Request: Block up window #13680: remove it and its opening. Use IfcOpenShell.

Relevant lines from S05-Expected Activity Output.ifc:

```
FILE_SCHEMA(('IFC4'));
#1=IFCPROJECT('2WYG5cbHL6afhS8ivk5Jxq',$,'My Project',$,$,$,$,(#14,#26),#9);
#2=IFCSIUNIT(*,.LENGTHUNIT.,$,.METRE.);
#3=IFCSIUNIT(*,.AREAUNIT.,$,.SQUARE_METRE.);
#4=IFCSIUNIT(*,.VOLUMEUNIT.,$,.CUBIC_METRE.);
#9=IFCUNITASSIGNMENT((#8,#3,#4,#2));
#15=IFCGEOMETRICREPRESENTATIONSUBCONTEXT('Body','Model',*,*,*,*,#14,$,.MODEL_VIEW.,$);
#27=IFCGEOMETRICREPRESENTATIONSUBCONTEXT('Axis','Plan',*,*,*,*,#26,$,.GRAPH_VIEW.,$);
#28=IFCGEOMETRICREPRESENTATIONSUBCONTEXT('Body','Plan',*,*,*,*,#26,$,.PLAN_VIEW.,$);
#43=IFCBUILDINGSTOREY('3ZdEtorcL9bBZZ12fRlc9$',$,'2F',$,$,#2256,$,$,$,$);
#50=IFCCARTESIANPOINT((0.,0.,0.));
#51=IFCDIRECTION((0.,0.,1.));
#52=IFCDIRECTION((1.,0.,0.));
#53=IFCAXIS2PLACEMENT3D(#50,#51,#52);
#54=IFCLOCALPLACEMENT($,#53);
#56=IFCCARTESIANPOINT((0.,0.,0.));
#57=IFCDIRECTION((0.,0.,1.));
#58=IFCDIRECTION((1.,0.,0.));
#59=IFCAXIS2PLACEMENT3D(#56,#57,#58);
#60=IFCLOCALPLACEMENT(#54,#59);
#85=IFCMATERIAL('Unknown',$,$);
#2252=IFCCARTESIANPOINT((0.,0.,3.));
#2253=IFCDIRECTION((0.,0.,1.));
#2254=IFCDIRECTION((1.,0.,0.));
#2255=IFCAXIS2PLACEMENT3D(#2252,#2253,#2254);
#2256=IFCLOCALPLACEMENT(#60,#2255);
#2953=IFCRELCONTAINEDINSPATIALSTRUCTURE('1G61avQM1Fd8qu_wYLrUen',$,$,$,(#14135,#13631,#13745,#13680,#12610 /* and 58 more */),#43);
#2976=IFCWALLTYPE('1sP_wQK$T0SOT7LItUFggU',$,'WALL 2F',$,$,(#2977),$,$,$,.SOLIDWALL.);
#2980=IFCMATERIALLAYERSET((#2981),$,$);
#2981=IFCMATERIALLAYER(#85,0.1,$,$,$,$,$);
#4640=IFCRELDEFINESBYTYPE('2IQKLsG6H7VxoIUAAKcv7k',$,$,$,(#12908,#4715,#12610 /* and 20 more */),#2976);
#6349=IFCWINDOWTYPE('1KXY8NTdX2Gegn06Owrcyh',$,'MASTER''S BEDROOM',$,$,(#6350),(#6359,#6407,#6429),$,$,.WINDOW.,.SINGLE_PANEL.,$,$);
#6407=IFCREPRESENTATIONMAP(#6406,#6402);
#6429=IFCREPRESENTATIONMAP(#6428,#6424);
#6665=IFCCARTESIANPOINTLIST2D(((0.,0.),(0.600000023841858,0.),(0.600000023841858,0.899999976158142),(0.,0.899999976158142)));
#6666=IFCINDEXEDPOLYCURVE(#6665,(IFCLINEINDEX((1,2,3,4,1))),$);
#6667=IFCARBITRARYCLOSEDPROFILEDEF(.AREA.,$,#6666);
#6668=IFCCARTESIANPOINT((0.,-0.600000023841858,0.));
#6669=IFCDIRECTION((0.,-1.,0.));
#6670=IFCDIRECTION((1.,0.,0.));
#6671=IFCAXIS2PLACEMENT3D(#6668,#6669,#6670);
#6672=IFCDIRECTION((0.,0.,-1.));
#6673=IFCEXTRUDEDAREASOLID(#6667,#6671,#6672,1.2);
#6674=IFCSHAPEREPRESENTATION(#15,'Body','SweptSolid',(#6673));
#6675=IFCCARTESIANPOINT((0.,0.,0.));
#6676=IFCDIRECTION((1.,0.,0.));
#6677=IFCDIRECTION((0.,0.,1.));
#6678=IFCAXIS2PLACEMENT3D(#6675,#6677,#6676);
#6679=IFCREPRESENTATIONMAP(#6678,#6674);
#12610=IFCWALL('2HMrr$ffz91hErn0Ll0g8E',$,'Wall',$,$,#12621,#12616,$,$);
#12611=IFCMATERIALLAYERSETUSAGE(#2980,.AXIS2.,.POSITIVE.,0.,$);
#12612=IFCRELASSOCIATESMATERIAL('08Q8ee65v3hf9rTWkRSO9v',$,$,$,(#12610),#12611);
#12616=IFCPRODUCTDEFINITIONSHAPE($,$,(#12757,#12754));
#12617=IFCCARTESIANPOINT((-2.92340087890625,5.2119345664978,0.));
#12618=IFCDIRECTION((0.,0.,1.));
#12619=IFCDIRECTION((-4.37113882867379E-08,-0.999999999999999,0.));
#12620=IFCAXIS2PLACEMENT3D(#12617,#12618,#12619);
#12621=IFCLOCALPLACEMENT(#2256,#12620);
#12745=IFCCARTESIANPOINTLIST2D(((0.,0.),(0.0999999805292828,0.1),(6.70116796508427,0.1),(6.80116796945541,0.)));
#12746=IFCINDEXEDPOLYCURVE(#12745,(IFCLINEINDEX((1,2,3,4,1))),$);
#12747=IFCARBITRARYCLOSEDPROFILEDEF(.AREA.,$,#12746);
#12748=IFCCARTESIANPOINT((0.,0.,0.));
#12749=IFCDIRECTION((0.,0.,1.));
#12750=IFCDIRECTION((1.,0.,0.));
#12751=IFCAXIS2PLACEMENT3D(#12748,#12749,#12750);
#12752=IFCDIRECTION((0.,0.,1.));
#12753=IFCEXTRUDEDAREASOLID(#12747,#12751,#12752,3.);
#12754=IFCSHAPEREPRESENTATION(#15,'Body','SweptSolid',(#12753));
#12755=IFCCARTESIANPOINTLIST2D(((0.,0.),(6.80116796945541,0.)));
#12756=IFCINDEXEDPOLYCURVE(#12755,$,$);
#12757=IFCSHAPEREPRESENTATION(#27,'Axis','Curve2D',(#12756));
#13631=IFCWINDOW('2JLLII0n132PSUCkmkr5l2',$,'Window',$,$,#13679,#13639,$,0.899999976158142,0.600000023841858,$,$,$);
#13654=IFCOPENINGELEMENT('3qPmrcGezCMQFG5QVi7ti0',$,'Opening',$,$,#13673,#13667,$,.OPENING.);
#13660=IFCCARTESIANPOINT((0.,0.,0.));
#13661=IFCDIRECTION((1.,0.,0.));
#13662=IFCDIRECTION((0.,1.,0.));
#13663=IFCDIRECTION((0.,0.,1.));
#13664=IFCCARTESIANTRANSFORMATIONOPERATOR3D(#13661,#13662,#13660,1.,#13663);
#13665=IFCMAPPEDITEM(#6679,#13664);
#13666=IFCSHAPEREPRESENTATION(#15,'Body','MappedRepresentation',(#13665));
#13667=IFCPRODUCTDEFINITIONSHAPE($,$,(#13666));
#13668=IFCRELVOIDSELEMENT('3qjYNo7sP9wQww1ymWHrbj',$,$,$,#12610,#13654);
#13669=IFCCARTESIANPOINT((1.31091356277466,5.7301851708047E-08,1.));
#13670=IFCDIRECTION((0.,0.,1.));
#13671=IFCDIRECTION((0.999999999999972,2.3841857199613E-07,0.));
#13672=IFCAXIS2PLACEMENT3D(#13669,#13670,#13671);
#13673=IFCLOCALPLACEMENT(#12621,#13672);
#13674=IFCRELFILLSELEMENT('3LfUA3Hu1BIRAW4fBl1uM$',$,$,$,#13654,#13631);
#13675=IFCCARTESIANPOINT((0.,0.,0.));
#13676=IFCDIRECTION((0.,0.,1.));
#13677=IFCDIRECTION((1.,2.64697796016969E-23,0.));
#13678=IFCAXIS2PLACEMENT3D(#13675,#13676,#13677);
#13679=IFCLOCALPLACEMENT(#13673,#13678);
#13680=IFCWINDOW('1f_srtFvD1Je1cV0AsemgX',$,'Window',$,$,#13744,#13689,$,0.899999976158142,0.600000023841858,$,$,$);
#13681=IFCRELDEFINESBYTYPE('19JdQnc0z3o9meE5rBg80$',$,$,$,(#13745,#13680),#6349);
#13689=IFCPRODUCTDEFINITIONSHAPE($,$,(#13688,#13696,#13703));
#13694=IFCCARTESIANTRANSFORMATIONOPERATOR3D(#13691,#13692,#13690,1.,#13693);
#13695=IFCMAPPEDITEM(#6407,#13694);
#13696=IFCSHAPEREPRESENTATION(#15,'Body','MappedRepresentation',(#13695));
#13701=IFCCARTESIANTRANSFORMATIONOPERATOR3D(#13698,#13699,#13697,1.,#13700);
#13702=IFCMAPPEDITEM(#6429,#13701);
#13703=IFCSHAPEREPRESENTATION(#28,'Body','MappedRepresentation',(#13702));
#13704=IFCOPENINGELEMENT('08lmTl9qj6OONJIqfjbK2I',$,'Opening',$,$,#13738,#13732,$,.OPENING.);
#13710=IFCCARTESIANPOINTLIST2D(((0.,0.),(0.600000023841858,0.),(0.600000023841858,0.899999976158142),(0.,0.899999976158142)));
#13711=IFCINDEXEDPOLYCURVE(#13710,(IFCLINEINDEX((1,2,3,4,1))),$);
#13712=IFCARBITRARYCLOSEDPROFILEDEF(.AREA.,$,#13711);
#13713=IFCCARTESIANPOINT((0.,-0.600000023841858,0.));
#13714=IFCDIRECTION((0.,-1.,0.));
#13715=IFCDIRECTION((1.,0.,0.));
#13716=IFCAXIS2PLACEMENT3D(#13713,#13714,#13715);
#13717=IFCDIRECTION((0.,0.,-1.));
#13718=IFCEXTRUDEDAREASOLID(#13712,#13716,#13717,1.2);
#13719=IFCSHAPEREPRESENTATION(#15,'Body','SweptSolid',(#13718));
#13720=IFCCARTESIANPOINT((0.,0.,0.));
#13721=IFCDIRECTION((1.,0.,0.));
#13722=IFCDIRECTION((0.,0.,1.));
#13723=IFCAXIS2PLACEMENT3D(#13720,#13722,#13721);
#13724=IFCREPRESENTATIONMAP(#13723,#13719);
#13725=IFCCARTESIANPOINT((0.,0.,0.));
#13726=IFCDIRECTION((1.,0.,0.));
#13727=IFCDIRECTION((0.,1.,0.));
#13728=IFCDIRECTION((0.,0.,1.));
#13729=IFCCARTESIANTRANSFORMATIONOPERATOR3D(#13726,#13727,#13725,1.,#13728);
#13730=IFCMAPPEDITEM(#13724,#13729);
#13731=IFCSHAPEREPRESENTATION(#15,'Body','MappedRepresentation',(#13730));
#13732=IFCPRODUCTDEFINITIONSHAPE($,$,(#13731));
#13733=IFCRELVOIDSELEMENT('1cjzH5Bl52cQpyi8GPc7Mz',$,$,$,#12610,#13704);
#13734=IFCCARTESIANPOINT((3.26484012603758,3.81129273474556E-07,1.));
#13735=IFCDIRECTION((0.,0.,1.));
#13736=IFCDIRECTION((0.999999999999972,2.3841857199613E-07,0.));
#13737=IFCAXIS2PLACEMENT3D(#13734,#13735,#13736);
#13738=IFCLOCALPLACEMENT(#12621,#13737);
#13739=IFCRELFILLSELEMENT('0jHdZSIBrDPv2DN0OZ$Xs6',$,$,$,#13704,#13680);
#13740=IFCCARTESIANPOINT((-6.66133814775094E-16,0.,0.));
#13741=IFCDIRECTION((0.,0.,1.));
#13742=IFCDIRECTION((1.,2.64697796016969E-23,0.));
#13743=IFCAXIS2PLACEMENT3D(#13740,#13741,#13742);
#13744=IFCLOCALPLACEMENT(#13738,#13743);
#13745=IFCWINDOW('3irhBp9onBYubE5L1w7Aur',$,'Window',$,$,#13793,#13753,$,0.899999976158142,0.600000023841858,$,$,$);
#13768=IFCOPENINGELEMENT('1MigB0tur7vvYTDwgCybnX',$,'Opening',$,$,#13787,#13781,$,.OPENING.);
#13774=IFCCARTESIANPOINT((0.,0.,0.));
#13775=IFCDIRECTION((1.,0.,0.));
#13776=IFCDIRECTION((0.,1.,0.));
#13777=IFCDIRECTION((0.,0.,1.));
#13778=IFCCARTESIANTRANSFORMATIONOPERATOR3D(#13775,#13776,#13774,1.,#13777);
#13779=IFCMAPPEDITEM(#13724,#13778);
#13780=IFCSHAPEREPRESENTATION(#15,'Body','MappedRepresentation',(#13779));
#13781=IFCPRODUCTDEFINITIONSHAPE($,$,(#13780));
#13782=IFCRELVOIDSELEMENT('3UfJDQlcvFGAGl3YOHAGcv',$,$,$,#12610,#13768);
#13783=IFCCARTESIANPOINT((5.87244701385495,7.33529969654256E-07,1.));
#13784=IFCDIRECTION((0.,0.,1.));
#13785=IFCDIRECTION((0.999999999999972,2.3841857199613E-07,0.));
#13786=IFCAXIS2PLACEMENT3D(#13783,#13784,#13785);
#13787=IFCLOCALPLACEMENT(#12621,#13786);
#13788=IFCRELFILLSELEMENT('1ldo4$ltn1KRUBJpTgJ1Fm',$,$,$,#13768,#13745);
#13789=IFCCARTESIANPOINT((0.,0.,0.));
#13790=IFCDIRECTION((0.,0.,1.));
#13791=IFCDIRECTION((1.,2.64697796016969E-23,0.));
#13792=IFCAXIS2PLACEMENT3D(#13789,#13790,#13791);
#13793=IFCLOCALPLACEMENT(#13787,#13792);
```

```python
import ifcopenshell
import ifcopenshell.api.feature
import ifcopenshell.api.root
import ifcopenshell.geom
import ifcopenshell.util.shape

model = ifcopenshell.open("S05-Expected Activity Output.ifc")
settings = ifcopenshell.geom.settings()


def volume(element):
    """Net volume in cubic metres, openings subtracted."""
    shape = ifcopenshell.geom.create_shape(settings, element)
    return ifcopenshell.util.shape.get_volume(shape.geometry)


window = model.by_id(13680)
opening = window.FillsVoids[0].RelatingOpeningElement
wall = opening.VoidsElements[0].RelatingBuildingElement
before = volume(wall)

ifcopenshell.api.root.remove_product(model, product=window)
ifcopenshell.api.feature.remove_feature(model, feature=opening)

after = volume(wall)

print(f"wall volume {before:.3f} -> {after:.3f} m3")

model.write("S05-Expected Activity Output_edited.ifc")
```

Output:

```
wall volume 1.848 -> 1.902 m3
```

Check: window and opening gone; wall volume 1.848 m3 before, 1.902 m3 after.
